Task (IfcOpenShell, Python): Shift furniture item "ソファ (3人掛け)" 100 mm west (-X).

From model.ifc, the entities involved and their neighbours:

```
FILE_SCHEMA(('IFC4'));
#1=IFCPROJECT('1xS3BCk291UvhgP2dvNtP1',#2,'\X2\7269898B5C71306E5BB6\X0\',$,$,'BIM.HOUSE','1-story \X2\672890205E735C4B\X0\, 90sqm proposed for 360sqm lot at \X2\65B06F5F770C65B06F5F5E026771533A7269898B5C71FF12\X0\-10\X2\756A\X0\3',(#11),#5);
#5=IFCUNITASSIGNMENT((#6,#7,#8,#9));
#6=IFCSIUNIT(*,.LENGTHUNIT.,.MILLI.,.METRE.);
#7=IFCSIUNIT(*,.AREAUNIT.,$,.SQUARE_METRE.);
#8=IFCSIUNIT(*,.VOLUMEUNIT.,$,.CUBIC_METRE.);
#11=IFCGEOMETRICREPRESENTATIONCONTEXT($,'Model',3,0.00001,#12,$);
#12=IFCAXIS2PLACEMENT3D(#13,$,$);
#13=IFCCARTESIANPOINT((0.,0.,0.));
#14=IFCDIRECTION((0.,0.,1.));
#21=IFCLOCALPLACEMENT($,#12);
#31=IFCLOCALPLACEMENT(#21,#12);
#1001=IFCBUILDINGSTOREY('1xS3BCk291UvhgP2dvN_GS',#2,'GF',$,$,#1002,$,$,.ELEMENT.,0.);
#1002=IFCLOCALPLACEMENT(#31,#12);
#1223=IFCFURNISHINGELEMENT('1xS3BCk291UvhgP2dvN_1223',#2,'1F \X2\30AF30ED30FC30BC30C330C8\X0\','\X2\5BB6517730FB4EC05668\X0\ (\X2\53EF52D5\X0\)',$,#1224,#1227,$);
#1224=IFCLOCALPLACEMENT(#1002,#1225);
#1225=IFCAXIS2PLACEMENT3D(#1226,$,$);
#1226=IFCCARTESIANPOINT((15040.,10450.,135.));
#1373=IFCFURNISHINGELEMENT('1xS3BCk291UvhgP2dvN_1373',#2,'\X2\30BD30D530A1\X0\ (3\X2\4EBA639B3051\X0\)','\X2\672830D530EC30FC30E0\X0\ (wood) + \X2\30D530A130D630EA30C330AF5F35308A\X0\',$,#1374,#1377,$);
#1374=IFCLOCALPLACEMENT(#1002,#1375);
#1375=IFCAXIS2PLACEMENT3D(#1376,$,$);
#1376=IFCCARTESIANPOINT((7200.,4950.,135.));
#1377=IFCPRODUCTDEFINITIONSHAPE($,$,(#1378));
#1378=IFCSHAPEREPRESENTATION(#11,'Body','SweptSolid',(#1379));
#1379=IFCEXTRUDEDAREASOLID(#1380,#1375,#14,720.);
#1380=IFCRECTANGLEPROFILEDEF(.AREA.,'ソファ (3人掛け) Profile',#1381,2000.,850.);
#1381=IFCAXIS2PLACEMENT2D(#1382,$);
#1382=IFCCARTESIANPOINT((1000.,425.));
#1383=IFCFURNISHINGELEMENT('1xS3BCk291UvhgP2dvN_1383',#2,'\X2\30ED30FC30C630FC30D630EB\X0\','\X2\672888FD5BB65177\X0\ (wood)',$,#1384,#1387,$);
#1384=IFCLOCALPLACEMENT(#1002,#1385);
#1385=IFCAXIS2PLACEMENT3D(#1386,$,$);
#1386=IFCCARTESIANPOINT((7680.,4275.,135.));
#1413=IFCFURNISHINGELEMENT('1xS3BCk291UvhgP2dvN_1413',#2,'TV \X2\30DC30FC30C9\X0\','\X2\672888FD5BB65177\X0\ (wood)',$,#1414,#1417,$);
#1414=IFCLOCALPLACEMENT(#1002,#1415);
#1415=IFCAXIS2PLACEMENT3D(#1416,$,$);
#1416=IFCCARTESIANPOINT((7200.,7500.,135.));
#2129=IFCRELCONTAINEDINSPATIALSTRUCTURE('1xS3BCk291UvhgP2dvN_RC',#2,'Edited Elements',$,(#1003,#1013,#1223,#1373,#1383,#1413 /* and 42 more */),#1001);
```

```python
import ifcopenshell
import ifcopenshell.api.geometry
import ifcopenshell.util.placement
import ifcopenshell.util.unit

model = ifcopenshell.open("model.ifc")
unit_scale = ifcopenshell.util.unit.calculate_unit_scale(model)

item = model.by_guid("1xS3BCk291UvhgP2dvN_1373")
matrix = ifcopenshell.util.placement.get_local_placement(item.ObjectPlacement)
matrix[0, 3] -= 0.1 / unit_scale
ifcopenshell.api.geometry.edit_object_placement(model, product=item, matrix=matrix, is_si=False)

print(ifcopenshell.util.placement.get_local_placement(item.ObjectPlacement).round(3) + 0.0)

model.write("model-out.ifc")
```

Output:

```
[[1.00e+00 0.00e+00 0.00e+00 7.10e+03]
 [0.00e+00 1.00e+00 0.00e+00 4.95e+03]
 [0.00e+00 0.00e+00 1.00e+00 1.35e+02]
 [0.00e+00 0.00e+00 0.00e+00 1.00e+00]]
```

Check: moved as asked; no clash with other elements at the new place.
